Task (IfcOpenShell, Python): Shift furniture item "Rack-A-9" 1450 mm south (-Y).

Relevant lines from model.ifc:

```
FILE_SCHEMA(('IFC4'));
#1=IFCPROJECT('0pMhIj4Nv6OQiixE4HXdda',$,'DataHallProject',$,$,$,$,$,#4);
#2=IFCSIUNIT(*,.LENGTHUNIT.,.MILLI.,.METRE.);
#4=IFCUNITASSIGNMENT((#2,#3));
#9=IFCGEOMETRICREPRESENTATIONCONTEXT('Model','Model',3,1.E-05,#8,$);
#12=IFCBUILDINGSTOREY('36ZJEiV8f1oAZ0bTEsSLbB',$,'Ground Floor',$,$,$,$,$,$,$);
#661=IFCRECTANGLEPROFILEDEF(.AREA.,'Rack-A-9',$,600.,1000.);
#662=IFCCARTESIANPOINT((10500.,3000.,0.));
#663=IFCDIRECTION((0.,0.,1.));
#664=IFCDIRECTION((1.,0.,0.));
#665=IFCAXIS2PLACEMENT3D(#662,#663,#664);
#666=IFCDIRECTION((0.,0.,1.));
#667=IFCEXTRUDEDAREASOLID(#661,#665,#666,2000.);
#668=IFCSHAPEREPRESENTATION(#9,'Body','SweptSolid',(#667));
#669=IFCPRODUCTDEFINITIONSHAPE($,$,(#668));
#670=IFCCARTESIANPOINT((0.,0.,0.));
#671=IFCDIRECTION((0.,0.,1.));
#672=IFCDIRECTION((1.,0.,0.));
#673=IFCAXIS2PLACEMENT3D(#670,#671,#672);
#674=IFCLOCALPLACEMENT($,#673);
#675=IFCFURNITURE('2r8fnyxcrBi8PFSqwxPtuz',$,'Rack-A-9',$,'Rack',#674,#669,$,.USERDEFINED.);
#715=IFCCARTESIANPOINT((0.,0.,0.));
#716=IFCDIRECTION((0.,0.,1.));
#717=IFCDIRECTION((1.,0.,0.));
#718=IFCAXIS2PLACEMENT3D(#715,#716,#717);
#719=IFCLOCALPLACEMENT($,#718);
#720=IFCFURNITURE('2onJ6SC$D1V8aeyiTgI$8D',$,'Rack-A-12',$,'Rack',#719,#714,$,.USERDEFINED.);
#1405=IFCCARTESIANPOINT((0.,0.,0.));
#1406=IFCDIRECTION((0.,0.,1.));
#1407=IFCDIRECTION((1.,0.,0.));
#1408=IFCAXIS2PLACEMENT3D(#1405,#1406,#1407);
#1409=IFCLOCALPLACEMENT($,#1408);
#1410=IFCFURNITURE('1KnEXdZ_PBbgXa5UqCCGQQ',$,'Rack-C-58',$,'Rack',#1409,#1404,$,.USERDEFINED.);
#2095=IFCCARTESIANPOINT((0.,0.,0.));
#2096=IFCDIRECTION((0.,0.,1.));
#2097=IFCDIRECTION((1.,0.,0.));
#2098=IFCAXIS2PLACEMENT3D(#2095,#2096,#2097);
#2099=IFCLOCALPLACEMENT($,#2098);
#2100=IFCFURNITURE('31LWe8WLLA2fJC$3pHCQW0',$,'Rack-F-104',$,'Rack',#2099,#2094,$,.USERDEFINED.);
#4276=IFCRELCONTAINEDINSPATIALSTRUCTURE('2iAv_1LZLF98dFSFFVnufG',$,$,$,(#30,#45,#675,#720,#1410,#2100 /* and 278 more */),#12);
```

```python
import ifcopenshell
import ifcopenshell.api.geometry
import ifcopenshell.util.placement
import ifcopenshell.util.unit

model = ifcopenshell.open("model.ifc")
unit_scale = ifcopenshell.util.unit.calculate_unit_scale(model)

item = model.by_guid("2r8fnyxcrBi8PFSqwxPtuz")
matrix = ifcopenshell.util.placement.get_local_placement(item.ObjectPlacement)
matrix[1, 3] -= 1.45 / unit_scale
ifcopenshell.api.geometry.edit_object_placement(model, product=item, matrix=matrix, is_si=False)

print(ifcopenshell.util.placement.get_local_placement(item.ObjectPlacement).round(3) + 0.0)

model.write("model_updated.ifc")
```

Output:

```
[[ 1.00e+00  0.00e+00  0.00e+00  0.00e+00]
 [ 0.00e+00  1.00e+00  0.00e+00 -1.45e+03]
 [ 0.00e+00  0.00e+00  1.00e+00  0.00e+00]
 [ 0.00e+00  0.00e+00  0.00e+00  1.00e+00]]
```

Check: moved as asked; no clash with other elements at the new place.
